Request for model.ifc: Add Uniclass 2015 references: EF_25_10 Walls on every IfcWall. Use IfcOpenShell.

First a look at what the model holds.

```python
import ifcopenshell

model = ifcopenshell.open("model.ifc")
print(model.schema)
print("classifications:", [c.Name for c in model.by_type("IfcClassification")])
for ifc_class in ("IfcDoor", "IfcRoof", "IfcStair", "IfcWall", "IfcWindow"):
    print(ifc_class, len(model.by_type(ifc_class)))
```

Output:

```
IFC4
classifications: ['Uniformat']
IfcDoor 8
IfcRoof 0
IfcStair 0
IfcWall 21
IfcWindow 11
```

```python
import ifcopenshell
import ifcopenshell.api.classification

model = ifcopenshell.open("model.ifc")

system = ifcopenshell.api.classification.add_classification(model, classification="Uniclass 2015")

codes = {
    "IfcWall": ("EF_25_10", "Walls"),
}
for ifc_class, (code, name) in codes.items():
    products = model.by_type(ifc_class)
    ifcopenshell.api.classification.add_reference(
        model, products=products, classification=system, identification=code, name=name
    )
    print(code, len(products))

model.write("model_v2.ifc")
```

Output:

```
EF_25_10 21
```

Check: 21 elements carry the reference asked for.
